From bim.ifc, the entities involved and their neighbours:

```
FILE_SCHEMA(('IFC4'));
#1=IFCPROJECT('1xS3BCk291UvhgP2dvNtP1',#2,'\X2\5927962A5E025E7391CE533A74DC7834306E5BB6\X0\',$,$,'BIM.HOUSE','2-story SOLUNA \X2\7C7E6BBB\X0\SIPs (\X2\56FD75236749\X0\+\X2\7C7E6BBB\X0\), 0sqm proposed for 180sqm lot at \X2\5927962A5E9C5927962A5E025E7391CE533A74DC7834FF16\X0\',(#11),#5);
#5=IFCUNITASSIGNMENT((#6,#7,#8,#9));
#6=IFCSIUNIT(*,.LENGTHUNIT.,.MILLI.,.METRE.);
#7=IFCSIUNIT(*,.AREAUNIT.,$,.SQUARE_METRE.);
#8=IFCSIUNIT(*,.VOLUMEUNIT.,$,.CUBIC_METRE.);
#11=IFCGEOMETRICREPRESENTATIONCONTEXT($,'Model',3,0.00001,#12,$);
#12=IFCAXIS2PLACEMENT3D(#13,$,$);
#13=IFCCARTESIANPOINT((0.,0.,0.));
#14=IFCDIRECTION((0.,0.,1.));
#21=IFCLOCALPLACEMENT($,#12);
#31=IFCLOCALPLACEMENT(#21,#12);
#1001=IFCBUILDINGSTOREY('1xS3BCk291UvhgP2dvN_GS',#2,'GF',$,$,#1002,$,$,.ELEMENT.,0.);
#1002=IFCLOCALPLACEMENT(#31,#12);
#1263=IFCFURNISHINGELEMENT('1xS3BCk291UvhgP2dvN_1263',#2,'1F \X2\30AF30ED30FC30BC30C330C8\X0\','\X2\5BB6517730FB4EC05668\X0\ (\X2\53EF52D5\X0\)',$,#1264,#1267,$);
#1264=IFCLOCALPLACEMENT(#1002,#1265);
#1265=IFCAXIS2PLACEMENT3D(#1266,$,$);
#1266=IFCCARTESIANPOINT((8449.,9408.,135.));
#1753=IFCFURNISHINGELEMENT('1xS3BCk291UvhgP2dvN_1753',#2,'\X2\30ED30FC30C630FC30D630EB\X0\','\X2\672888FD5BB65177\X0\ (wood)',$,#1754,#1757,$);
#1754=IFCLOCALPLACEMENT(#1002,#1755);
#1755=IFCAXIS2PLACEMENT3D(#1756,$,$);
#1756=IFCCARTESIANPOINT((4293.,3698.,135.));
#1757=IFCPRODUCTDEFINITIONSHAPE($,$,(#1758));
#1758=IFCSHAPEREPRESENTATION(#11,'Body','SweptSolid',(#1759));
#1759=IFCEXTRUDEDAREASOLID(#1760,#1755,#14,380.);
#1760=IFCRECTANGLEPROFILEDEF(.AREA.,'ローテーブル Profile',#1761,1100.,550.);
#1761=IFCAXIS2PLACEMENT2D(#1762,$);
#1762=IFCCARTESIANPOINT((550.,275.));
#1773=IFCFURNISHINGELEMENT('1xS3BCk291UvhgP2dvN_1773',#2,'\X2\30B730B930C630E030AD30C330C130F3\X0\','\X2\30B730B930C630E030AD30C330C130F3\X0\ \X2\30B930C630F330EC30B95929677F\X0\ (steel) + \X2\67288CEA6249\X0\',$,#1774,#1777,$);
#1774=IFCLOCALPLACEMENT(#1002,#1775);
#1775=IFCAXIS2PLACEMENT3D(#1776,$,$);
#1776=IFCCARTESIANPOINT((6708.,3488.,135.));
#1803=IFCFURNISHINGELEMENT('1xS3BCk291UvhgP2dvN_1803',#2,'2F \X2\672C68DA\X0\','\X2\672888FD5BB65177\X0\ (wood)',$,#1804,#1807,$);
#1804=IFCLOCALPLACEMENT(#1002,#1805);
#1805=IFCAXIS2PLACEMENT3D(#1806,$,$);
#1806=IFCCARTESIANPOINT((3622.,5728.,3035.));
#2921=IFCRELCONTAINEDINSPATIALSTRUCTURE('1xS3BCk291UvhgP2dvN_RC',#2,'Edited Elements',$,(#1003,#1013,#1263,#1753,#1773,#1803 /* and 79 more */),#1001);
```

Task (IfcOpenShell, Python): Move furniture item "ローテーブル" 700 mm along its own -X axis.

```python
import ifcopenshell
import ifcopenshell.api.geometry
import ifcopenshell.util.placement

model = ifcopenshell.open("bim.ifc")

item = model.by_guid("1xS3BCk291UvhgP2dvN_1753")
matrix = ifcopenshell.util.placement.get_local_placement(item.ObjectPlacement)
matrix[:3, 3] -= matrix[:3, 0] * 700.0
ifcopenshell.api.geometry.edit_object_placement(model, product=item, matrix=matrix, is_si=False)

print(ifcopenshell.util.placement.get_local_placement(item.ObjectPlacement).round(3) + 0.0)

model.write("bim_rev.ifc")
```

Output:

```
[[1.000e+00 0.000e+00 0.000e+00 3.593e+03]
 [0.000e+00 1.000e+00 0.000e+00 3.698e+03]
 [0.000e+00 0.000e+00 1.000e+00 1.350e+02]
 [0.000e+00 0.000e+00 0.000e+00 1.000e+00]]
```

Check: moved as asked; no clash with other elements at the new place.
